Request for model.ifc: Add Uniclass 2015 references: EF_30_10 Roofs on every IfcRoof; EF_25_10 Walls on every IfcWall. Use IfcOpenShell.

First a look at what the model holds.

```python
import ifcopenshell

model = ifcopenshell.open("model.ifc")
print(model.schema)
print("classifications:", [c.Name for c in model.by_type("IfcClassification")])
for ifc_class in ("IfcDoor", "IfcRoof", "IfcStair", "IfcWall", "IfcWindow"):
    print(ifc_class, len(model.by_type(ifc_class)))
```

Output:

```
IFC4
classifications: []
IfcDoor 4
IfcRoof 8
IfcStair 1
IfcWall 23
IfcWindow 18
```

```python
import ifcopenshell
import ifcopenshell.api.classification

model = ifcopenshell.open("model.ifc")

system = ifcopenshell.api.classification.add_classification(model, classification="Uniclass 2015")

codes = {
    "IfcRoof": ("EF_30_10", "Roofs"),
    "IfcWall": ("EF_25_10", "Walls"),
}
for ifc_class, (code, name) in codes.items():
    products = model.by_type(ifc_class)
    ifcopenshell.api.classification.add_reference(
        model, products=products, classification=system, identification=code, name=name
    )
    print(code, len(products))

model.write("model_rev.ifc")
```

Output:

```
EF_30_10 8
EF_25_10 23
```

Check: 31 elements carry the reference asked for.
